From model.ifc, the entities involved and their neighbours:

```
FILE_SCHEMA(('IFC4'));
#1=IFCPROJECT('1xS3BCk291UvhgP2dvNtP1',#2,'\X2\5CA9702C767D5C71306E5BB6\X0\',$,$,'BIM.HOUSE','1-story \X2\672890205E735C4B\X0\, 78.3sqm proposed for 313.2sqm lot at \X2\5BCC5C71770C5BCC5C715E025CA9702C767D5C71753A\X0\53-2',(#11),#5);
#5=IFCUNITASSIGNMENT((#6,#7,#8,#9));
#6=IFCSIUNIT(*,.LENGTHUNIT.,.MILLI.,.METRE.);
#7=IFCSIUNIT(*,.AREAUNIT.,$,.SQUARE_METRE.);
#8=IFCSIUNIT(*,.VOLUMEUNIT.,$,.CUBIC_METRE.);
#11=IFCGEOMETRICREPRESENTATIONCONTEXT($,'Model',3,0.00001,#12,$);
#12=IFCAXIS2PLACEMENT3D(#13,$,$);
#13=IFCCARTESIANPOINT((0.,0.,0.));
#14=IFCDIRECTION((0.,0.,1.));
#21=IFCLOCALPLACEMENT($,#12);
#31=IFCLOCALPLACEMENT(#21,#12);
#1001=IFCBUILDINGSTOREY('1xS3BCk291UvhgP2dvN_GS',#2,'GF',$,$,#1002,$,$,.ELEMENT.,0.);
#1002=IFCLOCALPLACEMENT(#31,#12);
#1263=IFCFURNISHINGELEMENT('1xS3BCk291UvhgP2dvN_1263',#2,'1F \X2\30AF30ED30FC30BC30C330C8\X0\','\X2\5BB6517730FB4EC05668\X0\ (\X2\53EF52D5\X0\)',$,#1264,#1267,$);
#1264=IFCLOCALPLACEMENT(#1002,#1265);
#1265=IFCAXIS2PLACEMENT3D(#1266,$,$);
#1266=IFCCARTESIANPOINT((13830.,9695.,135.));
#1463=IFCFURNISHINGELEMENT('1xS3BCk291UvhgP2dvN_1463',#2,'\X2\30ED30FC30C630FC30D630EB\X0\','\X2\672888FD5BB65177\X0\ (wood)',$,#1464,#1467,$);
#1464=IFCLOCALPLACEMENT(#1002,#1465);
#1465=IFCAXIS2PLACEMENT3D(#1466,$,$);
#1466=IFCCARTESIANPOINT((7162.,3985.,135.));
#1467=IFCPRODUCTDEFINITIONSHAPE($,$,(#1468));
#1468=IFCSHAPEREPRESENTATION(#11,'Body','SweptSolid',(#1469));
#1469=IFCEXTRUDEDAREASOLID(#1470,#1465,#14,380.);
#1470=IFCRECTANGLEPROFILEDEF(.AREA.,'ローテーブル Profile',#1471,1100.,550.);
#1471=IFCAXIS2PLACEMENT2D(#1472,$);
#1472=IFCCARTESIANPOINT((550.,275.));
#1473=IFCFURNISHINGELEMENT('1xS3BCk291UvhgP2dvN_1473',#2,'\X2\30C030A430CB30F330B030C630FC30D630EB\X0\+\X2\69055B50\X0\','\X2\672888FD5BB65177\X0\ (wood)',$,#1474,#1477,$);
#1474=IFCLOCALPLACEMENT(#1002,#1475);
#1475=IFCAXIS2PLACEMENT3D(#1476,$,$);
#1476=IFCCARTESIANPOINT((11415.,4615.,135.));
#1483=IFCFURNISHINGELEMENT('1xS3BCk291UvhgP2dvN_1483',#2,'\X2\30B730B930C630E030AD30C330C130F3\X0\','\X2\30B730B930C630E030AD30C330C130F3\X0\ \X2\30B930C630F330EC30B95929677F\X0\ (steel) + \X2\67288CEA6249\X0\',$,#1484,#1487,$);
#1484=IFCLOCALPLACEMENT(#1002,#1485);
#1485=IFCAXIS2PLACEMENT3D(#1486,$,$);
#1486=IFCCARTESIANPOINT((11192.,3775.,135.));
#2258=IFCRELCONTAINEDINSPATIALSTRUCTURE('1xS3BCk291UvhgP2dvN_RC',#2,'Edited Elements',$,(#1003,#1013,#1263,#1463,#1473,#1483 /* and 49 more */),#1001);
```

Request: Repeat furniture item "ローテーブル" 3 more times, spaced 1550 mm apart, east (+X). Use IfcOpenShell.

```python
import numpy as np
import ifcopenshell
import ifcopenshell.api.geometry
import ifcopenshell.api.root
import ifcopenshell.util.element
import ifcopenshell.util.placement
import ifcopenshell.util.unit

model = ifcopenshell.open("model.ifc")
unit_scale = ifcopenshell.util.unit.calculate_unit_scale(model)


def reuse_history(source, copy):
    """copy_class also copies each property set's owner history, people and application; keep the originals."""
    for rel in copy.IsDefinedBy:
        if rel.is_a("IfcRelDefinesByProperties") and (history := rel.RelatingPropertyDefinition.OwnerHistory):
            rel.RelatingPropertyDefinition.OwnerHistory = source.OwnerHistory
            ifcopenshell.util.element.remove_deep2(model, history)


source = model.by_guid("1xS3BCk291UvhgP2dvN_1463")
base = ifcopenshell.util.placement.get_local_placement(source.ObjectPlacement)
step = np.array([1.0, 0.0, 0.0]) * 1.55 / unit_scale

for i in range(1, 4):
    copy = ifcopenshell.api.root.copy_class(model, product=source)
    copy.Representation = ifcopenshell.util.element.copy_deep(
        model, source.Representation, exclude=["IfcGeometricRepresentationContext", "IfcRepresentationMap"]
    )
    reuse_history(source, copy)
    matrix = base.copy()
    matrix[:3, 3] += i * step
    print("added at", matrix[:3, 3].round(3) + 0.0)
    ifcopenshell.api.geometry.edit_object_placement(model, product=copy, matrix=matrix, is_si=False)

model.write("model-out.ifc")
```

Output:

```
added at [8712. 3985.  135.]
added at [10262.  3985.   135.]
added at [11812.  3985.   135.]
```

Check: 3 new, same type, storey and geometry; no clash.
